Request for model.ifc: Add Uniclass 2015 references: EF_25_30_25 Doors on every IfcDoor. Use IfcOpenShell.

First a look at what the model holds.

```python
import ifcopenshell

model = ifcopenshell.open("model.ifc")
print(model.schema)
print("classifications:", [c.Name for c in model.by_type("IfcClassification")])
for ifc_class in ("IfcDoor", "IfcRoof", "IfcStair", "IfcWall", "IfcWindow"):
    print(ifc_class, len(model.by_type(ifc_class)))
```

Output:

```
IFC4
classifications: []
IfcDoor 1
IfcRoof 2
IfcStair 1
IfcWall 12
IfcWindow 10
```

```python
import ifcopenshell
import ifcopenshell.api.classification

model = ifcopenshell.open("model.ifc")

system = ifcopenshell.api.classification.add_classification(model, classification="Uniclass 2015")

codes = {
    "IfcDoor": ("EF_25_30_25", "Doors"),
}
for ifc_class, (code, name) in codes.items():
    products = model.by_type(ifc_class)
    ifcopenshell.api.classification.add_reference(
        model, products=products, classification=system, identification=code, name=name
    )
    print(code, len(products))

model.write("model_edited.ifc")
```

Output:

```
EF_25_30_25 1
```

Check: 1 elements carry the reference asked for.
